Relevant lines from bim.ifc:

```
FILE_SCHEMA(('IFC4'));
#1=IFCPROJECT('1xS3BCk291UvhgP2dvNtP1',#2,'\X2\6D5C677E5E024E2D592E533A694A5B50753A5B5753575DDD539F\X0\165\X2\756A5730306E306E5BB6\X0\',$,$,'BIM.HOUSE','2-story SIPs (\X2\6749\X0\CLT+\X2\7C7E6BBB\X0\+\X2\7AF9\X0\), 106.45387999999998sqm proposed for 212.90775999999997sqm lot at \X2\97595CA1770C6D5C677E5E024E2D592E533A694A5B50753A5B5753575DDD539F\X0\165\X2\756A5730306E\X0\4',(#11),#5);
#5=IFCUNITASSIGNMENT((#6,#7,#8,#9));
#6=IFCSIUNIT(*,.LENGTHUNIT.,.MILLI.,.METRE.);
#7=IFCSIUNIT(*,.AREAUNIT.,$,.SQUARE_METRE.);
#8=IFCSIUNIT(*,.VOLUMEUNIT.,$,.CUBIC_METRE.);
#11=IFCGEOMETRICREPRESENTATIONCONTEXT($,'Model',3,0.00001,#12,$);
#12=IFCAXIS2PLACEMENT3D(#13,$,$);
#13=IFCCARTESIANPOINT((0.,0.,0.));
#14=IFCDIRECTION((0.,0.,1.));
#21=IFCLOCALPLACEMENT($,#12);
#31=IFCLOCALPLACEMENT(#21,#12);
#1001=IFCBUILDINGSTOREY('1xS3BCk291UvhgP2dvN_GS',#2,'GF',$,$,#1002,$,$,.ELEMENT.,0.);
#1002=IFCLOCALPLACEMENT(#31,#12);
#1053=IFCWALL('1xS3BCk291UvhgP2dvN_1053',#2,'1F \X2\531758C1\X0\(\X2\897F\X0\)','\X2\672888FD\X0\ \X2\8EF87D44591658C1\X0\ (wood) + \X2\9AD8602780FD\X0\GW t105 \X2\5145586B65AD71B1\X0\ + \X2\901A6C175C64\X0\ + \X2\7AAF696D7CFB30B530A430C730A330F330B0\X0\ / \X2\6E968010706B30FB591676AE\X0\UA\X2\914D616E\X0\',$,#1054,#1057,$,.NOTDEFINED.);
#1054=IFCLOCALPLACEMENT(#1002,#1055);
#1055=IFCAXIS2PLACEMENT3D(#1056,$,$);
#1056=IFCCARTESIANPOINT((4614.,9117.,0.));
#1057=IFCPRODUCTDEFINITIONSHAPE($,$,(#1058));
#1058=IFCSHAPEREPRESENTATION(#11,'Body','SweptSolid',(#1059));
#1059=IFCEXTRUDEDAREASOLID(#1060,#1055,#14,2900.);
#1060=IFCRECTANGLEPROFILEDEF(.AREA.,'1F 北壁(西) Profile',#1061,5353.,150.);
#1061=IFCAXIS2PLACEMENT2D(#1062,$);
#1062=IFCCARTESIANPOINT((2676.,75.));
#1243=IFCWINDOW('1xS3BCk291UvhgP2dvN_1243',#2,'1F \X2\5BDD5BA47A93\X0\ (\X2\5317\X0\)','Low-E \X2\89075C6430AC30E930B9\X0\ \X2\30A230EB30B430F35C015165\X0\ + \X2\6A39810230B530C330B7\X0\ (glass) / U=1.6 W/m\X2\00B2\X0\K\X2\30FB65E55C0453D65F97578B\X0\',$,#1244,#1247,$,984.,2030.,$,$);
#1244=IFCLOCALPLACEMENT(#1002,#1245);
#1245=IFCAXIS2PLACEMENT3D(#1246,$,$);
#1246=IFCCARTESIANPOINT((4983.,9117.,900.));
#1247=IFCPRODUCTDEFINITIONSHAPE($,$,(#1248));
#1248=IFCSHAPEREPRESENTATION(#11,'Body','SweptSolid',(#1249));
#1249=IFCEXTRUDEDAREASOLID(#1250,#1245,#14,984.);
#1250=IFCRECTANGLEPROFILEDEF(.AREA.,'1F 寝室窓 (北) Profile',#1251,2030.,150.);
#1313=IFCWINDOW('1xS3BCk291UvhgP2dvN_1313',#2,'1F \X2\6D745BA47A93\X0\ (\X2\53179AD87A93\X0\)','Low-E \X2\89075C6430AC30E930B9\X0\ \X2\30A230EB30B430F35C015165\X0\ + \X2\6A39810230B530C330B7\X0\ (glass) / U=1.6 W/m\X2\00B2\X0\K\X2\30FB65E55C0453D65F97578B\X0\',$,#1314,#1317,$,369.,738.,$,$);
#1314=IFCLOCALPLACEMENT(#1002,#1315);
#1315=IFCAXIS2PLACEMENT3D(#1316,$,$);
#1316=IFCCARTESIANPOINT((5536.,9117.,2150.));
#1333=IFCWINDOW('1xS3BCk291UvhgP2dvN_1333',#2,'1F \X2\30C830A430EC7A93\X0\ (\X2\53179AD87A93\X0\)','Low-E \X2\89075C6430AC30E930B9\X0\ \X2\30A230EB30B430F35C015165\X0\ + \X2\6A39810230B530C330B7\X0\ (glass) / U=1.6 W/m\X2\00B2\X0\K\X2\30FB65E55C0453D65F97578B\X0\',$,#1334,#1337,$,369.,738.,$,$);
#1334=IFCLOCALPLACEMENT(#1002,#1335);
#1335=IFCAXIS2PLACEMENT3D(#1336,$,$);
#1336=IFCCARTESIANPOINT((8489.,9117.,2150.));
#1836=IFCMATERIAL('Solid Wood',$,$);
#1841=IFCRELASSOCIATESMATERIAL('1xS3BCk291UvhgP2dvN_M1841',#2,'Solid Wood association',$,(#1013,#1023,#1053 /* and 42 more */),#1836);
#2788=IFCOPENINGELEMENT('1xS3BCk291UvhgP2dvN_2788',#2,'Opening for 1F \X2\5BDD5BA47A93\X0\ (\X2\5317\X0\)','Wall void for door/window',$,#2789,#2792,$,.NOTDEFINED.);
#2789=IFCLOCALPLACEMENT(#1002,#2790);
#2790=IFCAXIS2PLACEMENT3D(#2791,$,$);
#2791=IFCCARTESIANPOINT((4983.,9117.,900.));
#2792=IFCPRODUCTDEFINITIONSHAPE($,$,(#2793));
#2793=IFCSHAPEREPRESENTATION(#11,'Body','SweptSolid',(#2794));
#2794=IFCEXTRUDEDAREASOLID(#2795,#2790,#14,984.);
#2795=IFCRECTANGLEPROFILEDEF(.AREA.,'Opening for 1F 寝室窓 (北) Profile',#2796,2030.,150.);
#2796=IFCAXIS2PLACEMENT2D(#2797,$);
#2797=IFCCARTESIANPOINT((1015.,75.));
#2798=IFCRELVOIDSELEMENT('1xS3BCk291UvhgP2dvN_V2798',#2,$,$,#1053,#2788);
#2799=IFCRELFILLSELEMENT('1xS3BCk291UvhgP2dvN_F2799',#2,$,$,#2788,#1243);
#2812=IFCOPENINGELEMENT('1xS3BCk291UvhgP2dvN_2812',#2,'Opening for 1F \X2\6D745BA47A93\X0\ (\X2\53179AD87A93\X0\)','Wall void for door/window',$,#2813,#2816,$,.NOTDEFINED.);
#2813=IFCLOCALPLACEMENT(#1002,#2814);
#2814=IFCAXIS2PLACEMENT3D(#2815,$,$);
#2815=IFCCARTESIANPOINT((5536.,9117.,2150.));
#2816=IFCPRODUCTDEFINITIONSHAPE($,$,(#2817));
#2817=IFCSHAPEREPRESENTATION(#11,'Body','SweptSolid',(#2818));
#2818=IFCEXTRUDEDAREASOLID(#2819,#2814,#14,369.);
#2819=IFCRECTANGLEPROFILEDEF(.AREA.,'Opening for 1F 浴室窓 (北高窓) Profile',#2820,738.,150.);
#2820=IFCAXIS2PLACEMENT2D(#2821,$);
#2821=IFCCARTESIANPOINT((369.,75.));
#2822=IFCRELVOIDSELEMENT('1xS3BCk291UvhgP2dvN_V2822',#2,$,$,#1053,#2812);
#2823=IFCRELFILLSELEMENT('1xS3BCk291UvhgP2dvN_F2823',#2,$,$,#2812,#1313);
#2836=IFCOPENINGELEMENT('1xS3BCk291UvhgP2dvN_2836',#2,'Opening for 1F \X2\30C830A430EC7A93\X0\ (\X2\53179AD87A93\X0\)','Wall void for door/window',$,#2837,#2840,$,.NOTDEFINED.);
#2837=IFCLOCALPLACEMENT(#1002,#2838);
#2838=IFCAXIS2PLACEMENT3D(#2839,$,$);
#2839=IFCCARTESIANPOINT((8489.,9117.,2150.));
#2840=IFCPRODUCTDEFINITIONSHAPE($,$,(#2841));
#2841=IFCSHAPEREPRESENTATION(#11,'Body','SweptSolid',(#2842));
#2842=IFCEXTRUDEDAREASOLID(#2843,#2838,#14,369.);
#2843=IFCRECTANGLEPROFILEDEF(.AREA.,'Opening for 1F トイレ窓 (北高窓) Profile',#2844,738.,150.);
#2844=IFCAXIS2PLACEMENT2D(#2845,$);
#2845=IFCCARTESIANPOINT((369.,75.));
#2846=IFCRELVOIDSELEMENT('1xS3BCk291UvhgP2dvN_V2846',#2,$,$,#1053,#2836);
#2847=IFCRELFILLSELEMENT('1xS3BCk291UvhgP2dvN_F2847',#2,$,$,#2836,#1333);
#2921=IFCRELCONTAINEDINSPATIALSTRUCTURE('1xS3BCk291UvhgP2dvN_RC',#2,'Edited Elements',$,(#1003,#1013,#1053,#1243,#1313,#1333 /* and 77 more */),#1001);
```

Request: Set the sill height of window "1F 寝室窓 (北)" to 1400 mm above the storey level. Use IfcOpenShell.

```python
import numpy as np
import ifcopenshell
import ifcopenshell.api.geometry
import ifcopenshell.geom
import ifcopenshell.util.element
import ifcopenshell.util.placement
import ifcopenshell.util.shape
import ifcopenshell.util.unit

model = ifcopenshell.open("bim.ifc")
unit_scale = ifcopenshell.util.unit.calculate_unit_scale(model)

window = model.by_guid("1xS3BCk291UvhgP2dvN_1243")
opening = window.FillsVoids[0].RelatingOpeningElement
storey = ifcopenshell.util.element.get_container(window, ifc_class="IfcBuildingStorey")
level = ifcopenshell.util.placement.get_local_placement(storey.ObjectPlacement)[2, 3]

# The opening's origin need not be at the sill, so measure its lowest point.
shape = ifcopenshell.geom.create_shape(ifcopenshell.geom.settings(), opening)
bottom = ifcopenshell.util.shape.get_shape_bottom_elevation(shape, shape.geometry) / unit_scale
dz = level + 1400.0 - bottom

shift = np.array([0.0, 0.0, dz])
# The window is not placed relative to its opening, so move both.
for product in (opening, window):
    matrix = ifcopenshell.util.placement.get_local_placement(product.ObjectPlacement)
    matrix[:3, 3] += shift
    ifcopenshell.api.geometry.edit_object_placement(model, product=product, matrix=matrix, is_si=False)

print(f"moved by {dz * unit_scale:+.3f} m")

model.write("bim_rev.ifc")
```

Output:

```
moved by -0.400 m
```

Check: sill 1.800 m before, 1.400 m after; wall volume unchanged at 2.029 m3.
